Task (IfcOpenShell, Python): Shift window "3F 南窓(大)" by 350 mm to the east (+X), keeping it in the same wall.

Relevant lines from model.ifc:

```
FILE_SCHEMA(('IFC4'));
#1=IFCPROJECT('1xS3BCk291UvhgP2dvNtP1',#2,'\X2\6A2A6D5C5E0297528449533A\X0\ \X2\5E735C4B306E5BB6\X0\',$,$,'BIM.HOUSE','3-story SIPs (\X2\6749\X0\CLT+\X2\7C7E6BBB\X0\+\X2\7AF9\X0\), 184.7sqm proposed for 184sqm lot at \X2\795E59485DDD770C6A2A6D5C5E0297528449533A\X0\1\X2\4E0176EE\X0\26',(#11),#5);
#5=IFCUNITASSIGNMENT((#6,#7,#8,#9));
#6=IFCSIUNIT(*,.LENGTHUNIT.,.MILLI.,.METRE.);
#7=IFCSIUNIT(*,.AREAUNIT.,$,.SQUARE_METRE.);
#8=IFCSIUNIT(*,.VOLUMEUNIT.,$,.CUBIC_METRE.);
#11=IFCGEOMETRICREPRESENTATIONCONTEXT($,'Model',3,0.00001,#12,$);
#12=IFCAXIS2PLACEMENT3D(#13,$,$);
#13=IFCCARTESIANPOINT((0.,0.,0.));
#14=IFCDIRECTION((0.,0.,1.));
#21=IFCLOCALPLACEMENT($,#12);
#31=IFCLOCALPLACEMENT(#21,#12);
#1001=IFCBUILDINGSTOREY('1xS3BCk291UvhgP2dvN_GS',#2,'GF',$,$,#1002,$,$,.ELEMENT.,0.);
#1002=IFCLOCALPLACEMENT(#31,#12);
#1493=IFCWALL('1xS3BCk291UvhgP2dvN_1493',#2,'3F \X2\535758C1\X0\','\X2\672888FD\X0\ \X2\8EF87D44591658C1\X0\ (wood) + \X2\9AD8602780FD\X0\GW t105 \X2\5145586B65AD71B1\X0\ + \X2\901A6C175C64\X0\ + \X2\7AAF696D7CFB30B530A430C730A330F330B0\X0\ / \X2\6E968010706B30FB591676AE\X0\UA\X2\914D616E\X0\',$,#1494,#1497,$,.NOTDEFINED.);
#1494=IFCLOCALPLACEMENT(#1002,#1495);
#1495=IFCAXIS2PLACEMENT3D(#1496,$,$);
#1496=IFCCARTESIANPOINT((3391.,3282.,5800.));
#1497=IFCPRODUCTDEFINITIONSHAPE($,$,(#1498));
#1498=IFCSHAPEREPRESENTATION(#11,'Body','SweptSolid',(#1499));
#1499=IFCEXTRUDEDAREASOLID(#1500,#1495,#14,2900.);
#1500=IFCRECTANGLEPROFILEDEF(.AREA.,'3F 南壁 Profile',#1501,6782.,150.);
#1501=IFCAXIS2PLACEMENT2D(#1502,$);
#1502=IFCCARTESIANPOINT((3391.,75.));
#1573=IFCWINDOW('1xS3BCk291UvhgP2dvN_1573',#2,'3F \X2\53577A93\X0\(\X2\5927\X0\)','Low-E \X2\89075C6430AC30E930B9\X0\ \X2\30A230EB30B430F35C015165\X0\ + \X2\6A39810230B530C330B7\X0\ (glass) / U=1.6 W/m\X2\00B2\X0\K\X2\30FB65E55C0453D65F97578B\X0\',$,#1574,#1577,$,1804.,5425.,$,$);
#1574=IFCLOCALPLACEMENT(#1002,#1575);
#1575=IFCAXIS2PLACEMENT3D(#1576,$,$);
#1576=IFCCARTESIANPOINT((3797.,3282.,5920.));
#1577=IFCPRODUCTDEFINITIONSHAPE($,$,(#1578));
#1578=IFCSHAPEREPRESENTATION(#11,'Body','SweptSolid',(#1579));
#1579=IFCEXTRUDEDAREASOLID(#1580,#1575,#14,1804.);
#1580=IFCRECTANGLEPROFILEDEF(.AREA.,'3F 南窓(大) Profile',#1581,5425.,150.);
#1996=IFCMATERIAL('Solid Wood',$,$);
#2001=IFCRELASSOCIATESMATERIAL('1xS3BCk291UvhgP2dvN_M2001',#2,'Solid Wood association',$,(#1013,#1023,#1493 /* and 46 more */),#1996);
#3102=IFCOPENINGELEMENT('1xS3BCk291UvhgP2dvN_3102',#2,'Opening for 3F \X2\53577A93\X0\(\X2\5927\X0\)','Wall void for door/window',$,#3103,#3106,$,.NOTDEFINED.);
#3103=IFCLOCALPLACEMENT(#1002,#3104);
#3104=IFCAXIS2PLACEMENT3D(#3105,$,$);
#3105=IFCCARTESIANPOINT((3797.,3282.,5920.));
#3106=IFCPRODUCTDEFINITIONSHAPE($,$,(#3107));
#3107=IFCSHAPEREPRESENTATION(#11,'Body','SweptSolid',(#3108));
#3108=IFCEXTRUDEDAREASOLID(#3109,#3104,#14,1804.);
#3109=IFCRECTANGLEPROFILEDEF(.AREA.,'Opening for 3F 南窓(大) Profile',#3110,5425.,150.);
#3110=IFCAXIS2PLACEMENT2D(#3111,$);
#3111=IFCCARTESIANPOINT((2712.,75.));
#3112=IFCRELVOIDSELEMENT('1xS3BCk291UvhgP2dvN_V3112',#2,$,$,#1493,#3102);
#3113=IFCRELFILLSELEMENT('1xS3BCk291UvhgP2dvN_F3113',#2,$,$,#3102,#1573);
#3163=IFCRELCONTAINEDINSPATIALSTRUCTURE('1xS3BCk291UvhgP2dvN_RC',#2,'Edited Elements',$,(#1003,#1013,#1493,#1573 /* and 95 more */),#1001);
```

```python
import ifcopenshell
import ifcopenshell.api.geometry
import ifcopenshell.util.placement

model = ifcopenshell.open("model.ifc")

window = model.by_guid("1xS3BCk291UvhgP2dvN_1573")
opening = window.FillsVoids[0].RelatingOpeningElement
wall = opening.VoidsElements[0].RelatingBuildingElement

wall_matrix = ifcopenshell.util.placement.get_local_placement(wall.ObjectPlacement)
shift = wall_matrix[:3, 0] * 350.0
before = ifcopenshell.util.placement.get_local_placement(window.ObjectPlacement)[:3, 3].copy()

# The window is not placed relative to its opening, so move both.
for product in (opening, window):
    matrix = ifcopenshell.util.placement.get_local_placement(product.ObjectPlacement)
    matrix[:3, 3] += shift
    ifcopenshell.api.geometry.edit_object_placement(model, product=product, matrix=matrix, is_si=False)

after = ifcopenshell.util.placement.get_local_placement(window.ObjectPlacement)[:3, 3]
print("window moved by", (after - before).round(3) + 0.0)

model.write("model_v2.ifc")
```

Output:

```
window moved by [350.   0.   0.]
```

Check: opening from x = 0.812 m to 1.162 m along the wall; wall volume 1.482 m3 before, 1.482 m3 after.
